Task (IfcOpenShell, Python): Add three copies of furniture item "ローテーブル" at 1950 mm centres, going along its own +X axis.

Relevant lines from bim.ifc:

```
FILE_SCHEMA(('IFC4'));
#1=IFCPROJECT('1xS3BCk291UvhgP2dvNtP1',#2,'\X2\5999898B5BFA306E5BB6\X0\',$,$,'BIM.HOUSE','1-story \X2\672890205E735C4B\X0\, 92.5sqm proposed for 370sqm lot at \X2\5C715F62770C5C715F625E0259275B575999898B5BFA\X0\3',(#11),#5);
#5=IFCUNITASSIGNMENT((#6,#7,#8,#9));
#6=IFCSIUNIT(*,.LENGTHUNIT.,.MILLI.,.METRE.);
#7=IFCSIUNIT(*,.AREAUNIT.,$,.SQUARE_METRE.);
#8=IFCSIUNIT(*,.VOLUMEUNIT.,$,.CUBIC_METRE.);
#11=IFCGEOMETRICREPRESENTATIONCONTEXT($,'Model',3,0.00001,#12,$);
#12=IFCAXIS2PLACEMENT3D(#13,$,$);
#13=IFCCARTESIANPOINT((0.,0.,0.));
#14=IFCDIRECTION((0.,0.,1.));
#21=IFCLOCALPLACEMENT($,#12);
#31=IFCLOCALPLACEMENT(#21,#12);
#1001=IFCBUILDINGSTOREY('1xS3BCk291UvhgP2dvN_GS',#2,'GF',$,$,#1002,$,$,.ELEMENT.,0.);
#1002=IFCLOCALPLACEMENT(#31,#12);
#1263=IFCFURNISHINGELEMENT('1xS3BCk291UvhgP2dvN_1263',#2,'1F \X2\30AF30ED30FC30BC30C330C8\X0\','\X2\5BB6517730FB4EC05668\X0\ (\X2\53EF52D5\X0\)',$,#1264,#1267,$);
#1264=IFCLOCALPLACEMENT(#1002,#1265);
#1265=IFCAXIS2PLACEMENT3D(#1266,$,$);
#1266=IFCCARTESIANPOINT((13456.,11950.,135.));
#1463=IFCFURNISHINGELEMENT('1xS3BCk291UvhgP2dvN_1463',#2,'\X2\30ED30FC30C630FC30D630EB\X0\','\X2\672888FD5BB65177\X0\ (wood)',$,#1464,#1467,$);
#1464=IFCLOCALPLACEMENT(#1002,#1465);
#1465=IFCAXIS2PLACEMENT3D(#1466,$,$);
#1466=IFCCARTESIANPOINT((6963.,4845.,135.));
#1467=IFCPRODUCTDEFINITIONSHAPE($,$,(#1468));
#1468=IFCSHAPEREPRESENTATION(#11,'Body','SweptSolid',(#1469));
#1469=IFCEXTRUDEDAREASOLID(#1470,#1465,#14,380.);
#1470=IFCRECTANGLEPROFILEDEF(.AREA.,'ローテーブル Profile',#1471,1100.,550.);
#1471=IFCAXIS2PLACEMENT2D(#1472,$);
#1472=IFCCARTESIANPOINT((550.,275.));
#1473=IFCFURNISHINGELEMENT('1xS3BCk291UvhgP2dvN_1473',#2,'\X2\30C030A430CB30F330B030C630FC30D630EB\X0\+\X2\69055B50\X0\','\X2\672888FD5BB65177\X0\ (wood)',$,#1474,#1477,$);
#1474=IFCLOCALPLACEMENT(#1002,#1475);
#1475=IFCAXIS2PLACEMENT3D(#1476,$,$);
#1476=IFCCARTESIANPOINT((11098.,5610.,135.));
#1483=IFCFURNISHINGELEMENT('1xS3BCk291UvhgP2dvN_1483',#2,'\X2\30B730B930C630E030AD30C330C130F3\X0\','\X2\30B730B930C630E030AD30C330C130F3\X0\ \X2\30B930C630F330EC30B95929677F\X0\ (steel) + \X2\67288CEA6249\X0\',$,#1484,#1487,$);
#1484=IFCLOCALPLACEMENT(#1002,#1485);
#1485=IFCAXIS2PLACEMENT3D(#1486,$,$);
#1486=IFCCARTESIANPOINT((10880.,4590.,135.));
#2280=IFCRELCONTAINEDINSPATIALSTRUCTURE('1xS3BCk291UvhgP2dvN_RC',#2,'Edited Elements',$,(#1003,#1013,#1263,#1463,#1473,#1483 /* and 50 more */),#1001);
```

```python
import ifcopenshell
import ifcopenshell.api.geometry
import ifcopenshell.api.root
import ifcopenshell.util.element
import ifcopenshell.util.placement

model = ifcopenshell.open("bim.ifc")


def reuse_history(source, copy):
    """copy_class also copies each property set's owner history, people and application; keep the originals."""
    for rel in copy.IsDefinedBy:
        if rel.is_a("IfcRelDefinesByProperties") and (history := rel.RelatingPropertyDefinition.OwnerHistory):
            rel.RelatingPropertyDefinition.OwnerHistory = source.OwnerHistory
            ifcopenshell.util.element.remove_deep2(model, history)


source = model.by_guid("1xS3BCk291UvhgP2dvN_1463")
base = ifcopenshell.util.placement.get_local_placement(source.ObjectPlacement)
step = base[:3, 0] * 1950.0

for i in range(1, 4):
    copy = ifcopenshell.api.root.copy_class(model, product=source)
    copy.Representation = ifcopenshell.util.element.copy_deep(
        model, source.Representation, exclude=["IfcGeometricRepresentationContext", "IfcRepresentationMap"]
    )
    reuse_history(source, copy)
    matrix = base.copy()
    matrix[:3, 3] += i * step
    print("added at", matrix[:3, 3].round(3) + 0.0)
    ifcopenshell.api.geometry.edit_object_placement(model, product=copy, matrix=matrix, is_si=False)

model.write("bim-out.ifc")
```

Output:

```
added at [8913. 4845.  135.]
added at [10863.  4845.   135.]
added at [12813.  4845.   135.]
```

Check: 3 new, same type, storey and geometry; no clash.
